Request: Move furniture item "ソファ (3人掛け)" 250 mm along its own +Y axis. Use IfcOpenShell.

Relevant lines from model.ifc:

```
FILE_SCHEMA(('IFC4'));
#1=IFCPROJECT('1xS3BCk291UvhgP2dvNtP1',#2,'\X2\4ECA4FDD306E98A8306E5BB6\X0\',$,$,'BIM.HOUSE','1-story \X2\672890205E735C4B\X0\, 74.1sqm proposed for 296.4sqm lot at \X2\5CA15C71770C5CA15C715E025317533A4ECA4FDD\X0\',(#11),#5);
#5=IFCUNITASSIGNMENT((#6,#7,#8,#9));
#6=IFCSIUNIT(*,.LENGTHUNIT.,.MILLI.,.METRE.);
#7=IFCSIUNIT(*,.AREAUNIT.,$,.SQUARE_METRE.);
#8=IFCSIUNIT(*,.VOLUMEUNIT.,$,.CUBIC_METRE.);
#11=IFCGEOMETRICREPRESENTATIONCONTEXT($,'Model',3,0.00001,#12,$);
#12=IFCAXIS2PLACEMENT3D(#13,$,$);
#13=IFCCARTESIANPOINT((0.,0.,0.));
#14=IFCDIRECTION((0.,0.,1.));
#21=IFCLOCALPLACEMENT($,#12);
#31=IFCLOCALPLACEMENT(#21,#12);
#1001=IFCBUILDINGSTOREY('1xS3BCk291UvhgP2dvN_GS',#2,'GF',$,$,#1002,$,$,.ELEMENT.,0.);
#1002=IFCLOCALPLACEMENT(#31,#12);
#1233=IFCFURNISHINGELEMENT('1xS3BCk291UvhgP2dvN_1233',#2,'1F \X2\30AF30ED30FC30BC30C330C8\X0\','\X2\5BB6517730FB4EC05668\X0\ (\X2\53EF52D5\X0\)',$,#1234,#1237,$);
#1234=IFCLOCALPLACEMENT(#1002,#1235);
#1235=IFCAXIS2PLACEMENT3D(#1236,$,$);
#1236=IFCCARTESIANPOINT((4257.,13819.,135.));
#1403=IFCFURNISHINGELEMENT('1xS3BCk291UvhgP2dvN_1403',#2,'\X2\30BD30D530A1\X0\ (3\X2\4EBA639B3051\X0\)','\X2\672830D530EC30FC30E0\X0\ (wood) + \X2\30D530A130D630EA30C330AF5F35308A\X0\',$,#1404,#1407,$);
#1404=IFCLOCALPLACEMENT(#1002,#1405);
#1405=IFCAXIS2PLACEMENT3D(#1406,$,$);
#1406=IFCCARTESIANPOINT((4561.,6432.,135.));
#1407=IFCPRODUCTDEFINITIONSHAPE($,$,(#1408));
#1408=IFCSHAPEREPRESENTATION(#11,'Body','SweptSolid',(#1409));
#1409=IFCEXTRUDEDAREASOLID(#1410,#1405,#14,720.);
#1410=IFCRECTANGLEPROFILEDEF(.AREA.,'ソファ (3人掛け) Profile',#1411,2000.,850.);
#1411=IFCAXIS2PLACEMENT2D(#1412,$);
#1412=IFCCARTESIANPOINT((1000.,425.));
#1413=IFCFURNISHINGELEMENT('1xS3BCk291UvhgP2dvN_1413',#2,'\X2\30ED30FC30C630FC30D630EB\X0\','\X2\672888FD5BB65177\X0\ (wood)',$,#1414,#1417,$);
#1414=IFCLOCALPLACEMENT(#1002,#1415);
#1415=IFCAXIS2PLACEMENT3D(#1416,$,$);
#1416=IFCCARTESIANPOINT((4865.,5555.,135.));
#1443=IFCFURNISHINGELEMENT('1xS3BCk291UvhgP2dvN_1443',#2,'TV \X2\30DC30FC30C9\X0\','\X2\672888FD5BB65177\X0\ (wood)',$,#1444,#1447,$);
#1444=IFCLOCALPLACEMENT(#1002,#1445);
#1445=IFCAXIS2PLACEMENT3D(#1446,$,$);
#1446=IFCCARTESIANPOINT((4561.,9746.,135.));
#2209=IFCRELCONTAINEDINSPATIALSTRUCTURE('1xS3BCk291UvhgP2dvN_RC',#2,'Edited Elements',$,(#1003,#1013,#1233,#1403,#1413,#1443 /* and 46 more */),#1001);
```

```python
import ifcopenshell
import ifcopenshell.api.geometry
import ifcopenshell.util.placement
import ifcopenshell.util.unit

model = ifcopenshell.open("model.ifc")
unit_scale = ifcopenshell.util.unit.calculate_unit_scale(model)

item = model.by_guid("1xS3BCk291UvhgP2dvN_1403")
matrix = ifcopenshell.util.placement.get_local_placement(item.ObjectPlacement)
matrix[:3, 3] += matrix[:3, 1] * 0.25 / unit_scale
ifcopenshell.api.geometry.edit_object_placement(model, product=item, matrix=matrix, is_si=False)

print(ifcopenshell.util.placement.get_local_placement(item.ObjectPlacement).round(3) + 0.0)

model.write("model_v2.ifc")
```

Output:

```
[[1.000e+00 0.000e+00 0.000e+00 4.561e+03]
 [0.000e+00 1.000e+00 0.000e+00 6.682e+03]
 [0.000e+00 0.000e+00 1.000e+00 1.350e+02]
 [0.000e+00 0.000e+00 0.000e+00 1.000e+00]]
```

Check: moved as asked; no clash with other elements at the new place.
